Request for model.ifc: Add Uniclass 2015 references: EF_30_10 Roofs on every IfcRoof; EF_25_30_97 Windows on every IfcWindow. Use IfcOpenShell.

First a look at what the model holds.

```python
import ifcopenshell

model = ifcopenshell.open("model.ifc")
print(model.schema)
print("classifications:", [c.Name for c in model.by_type("IfcClassification")])
for ifc_class in ("IfcDoor", "IfcRoof", "IfcStair", "IfcWall", "IfcWindow"):
    print(ifc_class, len(model.by_type(ifc_class)))
```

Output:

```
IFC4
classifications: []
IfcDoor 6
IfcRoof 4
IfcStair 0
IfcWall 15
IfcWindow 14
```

```python
import ifcopenshell
import ifcopenshell.api.classification

model = ifcopenshell.open("model.ifc")

system = ifcopenshell.api.classification.add_classification(model, classification="Uniclass 2015")

codes = {
    "IfcRoof": ("EF_30_10", "Roofs"),
    "IfcWindow": ("EF_25_30_97", "Windows"),
}
for ifc_class, (code, name) in codes.items():
    products = model.by_type(ifc_class)
    ifcopenshell.api.classification.add_reference(
        model, products=products, classification=system, identification=code, name=name
    )
    print(code, len(products))

model.write("model_updated.ifc")
```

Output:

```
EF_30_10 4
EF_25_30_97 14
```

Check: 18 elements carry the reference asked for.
